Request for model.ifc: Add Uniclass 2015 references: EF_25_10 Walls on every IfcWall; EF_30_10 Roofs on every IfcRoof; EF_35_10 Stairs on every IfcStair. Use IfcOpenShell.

First a look at what the model holds.

```python
import ifcopenshell

model = ifcopenshell.open("model.ifc")
print(model.schema)
print("classifications:", [c.Name for c in model.by_type("IfcClassification")])
for ifc_class in ("IfcDoor", "IfcRoof", "IfcStair", "IfcWall", "IfcWindow"):
    print(ifc_class, len(model.by_type(ifc_class)))
```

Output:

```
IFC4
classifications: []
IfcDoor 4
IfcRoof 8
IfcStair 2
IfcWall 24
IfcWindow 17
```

```python
import ifcopenshell
import ifcopenshell.api.classification

model = ifcopenshell.open("model.ifc")

system = ifcopenshell.api.classification.add_classification(model, classification="Uniclass 2015")

codes = {
    "IfcWall": ("EF_25_10", "Walls"),
    "IfcRoof": ("EF_30_10", "Roofs"),
    "IfcStair": ("EF_35_10", "Stairs"),
}
for ifc_class, (code, name) in codes.items():
    products = model.by_type(ifc_class)
    ifcopenshell.api.classification.add_reference(
        model, products=products, classification=system, identification=code, name=name
    )
    print(code, len(products))

model.write("model_edited.ifc")
```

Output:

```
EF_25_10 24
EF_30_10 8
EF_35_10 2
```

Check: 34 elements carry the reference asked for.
